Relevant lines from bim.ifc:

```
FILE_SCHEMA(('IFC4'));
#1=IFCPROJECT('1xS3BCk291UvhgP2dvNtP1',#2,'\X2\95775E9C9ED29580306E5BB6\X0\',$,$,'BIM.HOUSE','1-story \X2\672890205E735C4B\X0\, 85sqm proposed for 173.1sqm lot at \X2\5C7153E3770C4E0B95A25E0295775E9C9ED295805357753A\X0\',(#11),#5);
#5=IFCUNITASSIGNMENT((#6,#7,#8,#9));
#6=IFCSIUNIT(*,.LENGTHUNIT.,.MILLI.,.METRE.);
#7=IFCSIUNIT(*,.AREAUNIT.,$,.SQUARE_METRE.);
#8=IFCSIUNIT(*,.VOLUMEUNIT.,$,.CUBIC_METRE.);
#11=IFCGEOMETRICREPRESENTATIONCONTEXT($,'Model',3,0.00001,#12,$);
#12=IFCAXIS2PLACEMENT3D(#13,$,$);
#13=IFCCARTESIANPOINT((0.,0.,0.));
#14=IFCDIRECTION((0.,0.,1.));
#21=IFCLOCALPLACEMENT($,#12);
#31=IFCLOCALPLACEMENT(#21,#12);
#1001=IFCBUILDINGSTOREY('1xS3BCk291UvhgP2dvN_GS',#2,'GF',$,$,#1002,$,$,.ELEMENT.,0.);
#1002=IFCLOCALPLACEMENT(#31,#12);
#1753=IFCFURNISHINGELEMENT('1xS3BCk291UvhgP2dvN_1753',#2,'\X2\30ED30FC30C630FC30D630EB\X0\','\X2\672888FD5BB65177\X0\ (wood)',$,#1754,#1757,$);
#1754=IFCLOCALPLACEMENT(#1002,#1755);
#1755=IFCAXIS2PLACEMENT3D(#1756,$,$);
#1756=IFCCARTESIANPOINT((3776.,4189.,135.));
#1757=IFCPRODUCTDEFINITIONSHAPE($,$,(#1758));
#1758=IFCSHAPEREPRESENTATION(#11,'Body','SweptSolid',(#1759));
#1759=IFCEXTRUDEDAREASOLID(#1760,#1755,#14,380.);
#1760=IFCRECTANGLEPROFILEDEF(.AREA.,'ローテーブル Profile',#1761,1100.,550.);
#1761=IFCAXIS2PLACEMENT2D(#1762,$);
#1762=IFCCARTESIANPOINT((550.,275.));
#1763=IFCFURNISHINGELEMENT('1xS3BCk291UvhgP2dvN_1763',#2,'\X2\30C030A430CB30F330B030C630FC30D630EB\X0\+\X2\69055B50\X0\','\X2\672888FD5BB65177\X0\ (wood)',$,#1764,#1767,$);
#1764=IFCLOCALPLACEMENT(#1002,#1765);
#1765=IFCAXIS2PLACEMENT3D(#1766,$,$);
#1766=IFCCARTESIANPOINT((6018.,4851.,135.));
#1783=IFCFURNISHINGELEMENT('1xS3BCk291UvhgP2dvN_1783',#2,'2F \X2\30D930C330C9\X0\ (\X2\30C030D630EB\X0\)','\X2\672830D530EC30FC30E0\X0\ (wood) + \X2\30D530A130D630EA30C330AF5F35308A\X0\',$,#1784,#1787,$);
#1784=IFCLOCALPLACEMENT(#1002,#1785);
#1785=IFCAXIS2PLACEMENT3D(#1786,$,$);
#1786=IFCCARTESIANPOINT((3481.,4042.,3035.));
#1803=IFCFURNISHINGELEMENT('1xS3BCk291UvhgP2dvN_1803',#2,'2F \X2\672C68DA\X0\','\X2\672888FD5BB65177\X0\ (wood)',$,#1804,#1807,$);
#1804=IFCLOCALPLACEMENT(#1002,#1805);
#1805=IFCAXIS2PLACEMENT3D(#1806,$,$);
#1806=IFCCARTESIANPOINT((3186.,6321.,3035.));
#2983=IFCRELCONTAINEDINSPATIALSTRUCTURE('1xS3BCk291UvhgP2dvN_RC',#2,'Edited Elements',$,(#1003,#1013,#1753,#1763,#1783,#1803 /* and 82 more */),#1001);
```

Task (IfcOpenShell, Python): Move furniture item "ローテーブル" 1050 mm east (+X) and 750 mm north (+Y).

```python
import ifcopenshell
import ifcopenshell.api.geometry
import ifcopenshell.util.placement

model = ifcopenshell.open("bim.ifc")

item = model.by_guid("1xS3BCk291UvhgP2dvN_1753")
matrix = ifcopenshell.util.placement.get_local_placement(item.ObjectPlacement)
matrix[0, 3] += 1050.0
matrix[1, 3] += 750.0
ifcopenshell.api.geometry.edit_object_placement(model, product=item, matrix=matrix, is_si=False)

print(ifcopenshell.util.placement.get_local_placement(item.ObjectPlacement).round(3) + 0.0)

model.write("bim_v2.ifc")
```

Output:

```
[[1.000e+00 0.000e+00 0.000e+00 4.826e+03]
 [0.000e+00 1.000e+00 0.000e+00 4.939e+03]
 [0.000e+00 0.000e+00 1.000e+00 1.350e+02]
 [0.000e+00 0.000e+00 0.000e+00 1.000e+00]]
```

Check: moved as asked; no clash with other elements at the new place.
